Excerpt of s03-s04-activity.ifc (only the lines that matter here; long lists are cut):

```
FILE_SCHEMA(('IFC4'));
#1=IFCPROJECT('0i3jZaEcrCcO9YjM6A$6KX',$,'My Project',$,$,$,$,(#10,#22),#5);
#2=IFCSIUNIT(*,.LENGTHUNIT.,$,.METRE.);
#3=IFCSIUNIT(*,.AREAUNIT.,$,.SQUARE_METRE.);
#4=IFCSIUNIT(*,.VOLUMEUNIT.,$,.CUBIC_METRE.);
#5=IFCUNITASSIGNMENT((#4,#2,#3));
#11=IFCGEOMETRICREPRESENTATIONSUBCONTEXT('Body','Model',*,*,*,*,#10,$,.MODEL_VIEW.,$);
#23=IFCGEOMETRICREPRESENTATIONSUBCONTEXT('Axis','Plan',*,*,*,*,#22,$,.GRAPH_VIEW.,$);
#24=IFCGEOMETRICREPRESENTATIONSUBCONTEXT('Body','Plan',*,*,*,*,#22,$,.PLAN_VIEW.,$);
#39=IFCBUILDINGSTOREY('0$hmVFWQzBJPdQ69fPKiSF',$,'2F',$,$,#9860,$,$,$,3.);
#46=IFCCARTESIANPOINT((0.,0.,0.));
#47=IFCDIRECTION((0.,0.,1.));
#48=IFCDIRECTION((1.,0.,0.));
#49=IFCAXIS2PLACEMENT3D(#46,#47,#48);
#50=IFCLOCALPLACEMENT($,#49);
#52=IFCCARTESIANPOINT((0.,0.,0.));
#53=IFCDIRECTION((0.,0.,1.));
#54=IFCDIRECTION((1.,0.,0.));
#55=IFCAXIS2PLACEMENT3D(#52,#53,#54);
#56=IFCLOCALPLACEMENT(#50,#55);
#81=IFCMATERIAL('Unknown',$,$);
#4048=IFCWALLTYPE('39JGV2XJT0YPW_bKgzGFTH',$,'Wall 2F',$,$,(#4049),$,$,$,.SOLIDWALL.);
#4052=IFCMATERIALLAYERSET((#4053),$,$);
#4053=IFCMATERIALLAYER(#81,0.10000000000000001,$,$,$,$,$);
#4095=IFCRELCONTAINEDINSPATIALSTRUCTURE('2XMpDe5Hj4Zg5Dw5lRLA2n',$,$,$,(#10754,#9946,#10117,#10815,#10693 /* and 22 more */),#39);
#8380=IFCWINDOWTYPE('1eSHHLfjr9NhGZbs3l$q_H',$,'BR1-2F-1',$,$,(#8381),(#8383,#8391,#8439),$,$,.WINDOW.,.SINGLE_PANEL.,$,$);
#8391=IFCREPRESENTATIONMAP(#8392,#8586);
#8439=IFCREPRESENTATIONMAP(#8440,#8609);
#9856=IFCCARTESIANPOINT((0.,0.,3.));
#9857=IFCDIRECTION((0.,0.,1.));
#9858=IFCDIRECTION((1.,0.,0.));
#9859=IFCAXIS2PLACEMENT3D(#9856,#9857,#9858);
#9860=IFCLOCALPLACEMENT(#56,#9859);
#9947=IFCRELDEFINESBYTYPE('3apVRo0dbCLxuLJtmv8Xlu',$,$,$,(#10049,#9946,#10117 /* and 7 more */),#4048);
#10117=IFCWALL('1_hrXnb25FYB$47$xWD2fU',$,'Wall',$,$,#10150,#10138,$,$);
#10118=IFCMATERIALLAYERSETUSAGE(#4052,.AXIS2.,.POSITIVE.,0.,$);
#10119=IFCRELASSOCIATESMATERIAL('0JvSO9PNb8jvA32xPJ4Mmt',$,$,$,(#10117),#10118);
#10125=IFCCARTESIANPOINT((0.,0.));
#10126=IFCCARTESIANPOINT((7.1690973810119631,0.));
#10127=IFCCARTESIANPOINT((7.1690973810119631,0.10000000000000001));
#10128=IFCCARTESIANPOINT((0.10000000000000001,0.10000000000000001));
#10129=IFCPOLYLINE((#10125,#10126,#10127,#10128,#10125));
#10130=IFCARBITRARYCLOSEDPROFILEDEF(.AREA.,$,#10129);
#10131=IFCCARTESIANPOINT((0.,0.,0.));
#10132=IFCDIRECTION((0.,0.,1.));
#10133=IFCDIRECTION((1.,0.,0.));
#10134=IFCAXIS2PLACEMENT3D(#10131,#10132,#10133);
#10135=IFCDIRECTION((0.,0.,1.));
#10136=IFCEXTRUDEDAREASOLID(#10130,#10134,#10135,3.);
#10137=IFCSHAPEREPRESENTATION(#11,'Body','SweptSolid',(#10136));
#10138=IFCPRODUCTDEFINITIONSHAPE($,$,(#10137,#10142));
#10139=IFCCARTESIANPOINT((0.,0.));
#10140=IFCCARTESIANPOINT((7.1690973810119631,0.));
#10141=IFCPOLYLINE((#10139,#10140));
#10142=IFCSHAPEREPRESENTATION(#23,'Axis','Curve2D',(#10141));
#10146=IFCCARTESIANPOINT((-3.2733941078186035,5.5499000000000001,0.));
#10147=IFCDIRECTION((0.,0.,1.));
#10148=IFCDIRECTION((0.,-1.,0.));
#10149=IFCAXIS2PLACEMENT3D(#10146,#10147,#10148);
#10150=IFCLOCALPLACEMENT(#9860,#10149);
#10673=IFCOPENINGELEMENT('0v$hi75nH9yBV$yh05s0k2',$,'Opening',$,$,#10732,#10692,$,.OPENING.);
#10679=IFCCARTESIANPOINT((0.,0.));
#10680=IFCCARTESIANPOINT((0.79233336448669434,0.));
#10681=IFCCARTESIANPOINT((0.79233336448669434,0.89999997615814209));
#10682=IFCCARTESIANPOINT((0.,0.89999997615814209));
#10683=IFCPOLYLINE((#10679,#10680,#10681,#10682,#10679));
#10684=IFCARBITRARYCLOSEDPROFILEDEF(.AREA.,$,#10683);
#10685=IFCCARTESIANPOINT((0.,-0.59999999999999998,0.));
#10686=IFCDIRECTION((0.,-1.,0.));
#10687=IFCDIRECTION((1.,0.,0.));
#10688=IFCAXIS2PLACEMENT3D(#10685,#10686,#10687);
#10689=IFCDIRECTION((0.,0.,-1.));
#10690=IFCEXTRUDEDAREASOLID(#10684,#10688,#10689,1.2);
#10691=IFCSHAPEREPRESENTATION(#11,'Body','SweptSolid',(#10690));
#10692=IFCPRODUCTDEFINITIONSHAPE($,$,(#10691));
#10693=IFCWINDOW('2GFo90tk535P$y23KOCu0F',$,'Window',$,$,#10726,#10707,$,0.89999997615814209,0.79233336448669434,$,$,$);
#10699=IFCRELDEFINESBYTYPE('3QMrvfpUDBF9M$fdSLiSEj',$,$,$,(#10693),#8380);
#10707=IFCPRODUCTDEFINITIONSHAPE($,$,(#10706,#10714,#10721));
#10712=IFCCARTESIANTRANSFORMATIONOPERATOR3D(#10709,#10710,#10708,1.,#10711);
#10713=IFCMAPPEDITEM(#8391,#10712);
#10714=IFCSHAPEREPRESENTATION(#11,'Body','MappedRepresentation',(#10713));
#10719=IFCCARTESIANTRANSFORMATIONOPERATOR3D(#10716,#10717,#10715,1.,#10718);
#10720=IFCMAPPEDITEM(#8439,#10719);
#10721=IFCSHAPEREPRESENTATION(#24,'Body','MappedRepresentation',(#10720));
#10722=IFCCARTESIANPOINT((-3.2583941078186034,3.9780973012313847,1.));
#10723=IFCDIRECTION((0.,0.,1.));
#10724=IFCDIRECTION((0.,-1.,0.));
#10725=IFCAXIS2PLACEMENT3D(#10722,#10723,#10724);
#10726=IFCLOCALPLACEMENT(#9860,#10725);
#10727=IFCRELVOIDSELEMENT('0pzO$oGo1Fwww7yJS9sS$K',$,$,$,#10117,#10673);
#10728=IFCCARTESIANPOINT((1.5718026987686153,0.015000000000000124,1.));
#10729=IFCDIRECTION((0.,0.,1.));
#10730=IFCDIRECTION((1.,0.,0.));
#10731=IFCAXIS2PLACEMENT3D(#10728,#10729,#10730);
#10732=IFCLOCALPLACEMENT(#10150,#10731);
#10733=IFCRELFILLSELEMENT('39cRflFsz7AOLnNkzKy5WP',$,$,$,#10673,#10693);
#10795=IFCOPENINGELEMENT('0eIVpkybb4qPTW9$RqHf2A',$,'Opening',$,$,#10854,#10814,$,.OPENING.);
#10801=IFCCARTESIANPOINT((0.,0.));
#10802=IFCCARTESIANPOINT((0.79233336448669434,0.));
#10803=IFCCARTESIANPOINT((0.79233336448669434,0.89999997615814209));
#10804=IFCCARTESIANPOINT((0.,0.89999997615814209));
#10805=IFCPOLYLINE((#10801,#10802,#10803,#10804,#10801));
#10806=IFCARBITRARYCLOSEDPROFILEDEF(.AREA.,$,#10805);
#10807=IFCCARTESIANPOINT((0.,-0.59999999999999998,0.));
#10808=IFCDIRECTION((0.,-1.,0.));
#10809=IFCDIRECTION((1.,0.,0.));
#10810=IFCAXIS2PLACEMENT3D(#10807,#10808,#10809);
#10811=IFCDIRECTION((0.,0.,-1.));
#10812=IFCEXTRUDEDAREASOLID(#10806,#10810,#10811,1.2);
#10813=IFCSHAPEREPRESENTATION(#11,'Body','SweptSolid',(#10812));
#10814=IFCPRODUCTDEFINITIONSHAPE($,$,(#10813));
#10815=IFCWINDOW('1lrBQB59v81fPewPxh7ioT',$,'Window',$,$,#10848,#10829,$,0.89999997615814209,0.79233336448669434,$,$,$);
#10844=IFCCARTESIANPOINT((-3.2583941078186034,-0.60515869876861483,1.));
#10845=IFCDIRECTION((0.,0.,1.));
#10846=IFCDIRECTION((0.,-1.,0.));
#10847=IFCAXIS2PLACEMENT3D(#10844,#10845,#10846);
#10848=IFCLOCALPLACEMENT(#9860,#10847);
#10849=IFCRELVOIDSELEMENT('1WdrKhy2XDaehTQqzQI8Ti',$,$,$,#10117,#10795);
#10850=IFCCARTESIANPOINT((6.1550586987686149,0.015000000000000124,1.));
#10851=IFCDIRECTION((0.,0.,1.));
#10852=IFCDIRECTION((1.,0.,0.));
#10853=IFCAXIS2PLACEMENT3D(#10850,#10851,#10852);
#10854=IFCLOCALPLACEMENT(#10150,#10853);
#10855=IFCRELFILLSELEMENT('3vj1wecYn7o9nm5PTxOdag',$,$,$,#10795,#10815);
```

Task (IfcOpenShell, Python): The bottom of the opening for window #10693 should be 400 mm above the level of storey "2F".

```python
import numpy as np
import ifcopenshell
import ifcopenshell.api.geometry
import ifcopenshell.geom
import ifcopenshell.util.element
import ifcopenshell.util.placement
import ifcopenshell.util.shape
import ifcopenshell.util.unit

model = ifcopenshell.open("s03-s04-activity.ifc")
unit_scale = ifcopenshell.util.unit.calculate_unit_scale(model)

window = model.by_guid("2GFo90tk535P$y23KOCu0F")
opening = window.FillsVoids[0].RelatingOpeningElement
storey = ifcopenshell.util.element.get_container(window, ifc_class="IfcBuildingStorey")
level = ifcopenshell.util.placement.get_local_placement(storey.ObjectPlacement)[2, 3]

# The opening's origin need not be at the sill, so measure its lowest point.
shape = ifcopenshell.geom.create_shape(ifcopenshell.geom.settings(), opening)
bottom = ifcopenshell.util.shape.get_shape_bottom_elevation(shape, shape.geometry) / unit_scale
dz = level + 0.4 - bottom

shift = np.array([0.0, 0.0, dz])
# The window is not placed relative to its opening, so move both.
for product in (opening, window):
    matrix = ifcopenshell.util.placement.get_local_placement(product.ObjectPlacement)
    matrix[:3, 3] += shift
    ifcopenshell.api.geometry.edit_object_placement(model, product=product, matrix=matrix, is_si=False)

print(f"moved by {dz * unit_scale:+.3f} m")

model.write("s03-s04-activity_v2.ifc")
```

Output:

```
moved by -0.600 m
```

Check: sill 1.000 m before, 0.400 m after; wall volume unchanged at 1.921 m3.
